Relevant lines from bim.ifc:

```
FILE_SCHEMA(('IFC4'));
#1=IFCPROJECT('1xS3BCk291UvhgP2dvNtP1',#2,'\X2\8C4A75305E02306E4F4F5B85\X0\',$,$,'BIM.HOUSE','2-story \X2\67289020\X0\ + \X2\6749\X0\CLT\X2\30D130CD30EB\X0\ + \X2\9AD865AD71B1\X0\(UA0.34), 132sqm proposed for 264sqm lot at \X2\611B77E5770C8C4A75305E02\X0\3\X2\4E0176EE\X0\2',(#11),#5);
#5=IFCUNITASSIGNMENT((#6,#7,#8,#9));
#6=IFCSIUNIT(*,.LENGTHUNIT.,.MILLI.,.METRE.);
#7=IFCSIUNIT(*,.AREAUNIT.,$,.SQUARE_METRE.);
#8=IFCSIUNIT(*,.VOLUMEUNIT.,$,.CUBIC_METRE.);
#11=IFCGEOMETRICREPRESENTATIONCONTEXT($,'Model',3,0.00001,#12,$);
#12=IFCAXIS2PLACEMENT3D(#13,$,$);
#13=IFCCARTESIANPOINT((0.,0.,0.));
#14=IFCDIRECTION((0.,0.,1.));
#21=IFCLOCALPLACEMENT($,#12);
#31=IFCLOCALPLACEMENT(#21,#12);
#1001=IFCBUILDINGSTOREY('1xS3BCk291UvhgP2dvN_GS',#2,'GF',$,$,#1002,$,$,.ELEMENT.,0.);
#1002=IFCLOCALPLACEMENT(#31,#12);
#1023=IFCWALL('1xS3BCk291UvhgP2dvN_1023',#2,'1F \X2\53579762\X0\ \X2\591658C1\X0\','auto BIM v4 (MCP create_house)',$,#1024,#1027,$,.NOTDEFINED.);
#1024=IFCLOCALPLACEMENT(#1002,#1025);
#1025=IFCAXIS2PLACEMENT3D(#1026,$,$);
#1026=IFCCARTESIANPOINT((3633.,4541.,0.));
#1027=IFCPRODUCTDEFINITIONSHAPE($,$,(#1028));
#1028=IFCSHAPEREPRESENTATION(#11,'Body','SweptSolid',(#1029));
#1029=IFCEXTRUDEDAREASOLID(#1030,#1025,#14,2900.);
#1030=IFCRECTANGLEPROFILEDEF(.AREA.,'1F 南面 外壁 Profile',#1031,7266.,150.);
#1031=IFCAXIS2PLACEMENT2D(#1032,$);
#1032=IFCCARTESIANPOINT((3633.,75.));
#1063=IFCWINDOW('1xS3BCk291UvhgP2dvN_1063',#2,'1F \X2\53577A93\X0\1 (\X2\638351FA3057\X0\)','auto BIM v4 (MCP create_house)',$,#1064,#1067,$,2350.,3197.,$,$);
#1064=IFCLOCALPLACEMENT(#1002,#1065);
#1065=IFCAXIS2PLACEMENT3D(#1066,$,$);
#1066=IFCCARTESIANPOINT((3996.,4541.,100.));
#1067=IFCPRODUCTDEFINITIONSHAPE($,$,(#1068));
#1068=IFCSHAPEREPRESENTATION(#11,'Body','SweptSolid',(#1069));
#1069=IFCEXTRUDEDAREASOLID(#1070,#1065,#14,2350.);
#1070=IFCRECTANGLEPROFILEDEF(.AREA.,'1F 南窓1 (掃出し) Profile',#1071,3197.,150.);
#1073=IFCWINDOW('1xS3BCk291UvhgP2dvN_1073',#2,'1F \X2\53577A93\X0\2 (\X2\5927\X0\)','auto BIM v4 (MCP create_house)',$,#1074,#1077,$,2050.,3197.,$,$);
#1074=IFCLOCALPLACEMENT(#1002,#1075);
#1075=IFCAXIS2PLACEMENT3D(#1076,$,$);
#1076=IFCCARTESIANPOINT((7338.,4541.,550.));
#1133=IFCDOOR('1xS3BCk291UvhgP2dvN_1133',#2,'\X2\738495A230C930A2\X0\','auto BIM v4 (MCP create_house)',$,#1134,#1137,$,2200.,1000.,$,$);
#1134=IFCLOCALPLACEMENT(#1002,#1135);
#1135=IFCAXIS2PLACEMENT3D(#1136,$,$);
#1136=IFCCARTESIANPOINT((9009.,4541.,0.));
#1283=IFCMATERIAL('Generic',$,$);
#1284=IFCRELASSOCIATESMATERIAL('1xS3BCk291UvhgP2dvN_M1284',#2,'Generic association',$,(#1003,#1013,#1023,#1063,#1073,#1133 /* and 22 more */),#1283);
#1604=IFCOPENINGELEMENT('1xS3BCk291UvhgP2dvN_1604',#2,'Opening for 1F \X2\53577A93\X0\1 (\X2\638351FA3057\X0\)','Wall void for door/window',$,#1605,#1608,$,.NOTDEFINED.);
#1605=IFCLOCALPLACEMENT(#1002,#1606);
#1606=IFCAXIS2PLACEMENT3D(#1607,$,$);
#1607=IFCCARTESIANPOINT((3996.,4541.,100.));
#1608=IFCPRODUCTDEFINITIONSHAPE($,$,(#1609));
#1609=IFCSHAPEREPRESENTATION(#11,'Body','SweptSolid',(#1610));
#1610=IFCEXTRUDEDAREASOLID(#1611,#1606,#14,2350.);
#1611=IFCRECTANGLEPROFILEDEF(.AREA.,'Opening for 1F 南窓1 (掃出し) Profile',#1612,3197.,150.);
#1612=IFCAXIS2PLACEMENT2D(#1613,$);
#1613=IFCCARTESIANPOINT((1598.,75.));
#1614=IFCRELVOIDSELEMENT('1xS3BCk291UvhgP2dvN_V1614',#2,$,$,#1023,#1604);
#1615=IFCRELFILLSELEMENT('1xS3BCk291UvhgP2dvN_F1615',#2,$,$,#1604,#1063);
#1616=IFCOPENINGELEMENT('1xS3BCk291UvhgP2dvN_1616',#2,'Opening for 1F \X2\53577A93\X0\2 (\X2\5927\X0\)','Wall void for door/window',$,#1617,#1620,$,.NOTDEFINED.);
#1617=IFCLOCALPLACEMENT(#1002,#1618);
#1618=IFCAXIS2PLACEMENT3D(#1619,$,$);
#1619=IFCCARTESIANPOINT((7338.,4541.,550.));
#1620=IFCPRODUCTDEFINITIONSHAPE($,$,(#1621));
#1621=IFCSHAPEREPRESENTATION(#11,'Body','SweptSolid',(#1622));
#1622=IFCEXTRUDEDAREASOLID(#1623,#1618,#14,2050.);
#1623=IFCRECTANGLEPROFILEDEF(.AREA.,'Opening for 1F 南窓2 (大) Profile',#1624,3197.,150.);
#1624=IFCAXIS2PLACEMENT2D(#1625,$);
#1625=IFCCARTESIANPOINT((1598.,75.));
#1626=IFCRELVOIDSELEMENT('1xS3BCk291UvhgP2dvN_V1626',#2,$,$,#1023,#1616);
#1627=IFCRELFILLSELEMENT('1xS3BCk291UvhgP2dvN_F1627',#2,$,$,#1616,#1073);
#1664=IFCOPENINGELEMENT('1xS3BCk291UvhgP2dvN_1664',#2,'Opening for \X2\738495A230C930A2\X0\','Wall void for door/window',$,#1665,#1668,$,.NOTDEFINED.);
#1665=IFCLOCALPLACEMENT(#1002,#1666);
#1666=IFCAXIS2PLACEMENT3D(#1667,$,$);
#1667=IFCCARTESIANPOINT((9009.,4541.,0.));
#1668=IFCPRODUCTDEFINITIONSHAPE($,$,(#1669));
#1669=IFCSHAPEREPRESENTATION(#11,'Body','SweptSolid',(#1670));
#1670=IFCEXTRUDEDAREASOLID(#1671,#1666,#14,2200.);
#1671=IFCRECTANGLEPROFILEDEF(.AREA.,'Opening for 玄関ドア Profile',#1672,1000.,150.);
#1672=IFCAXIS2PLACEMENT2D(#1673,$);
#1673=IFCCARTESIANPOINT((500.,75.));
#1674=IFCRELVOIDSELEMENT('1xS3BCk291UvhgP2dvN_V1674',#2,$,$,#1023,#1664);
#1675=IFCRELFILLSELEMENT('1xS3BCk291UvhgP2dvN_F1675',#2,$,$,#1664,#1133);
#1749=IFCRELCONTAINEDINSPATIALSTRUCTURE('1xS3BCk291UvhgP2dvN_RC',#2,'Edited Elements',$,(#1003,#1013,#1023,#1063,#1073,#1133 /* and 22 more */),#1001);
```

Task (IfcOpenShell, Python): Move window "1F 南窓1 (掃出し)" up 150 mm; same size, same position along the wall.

```python
import numpy as np
import ifcopenshell
import ifcopenshell.api.geometry
import ifcopenshell.util.placement
import ifcopenshell.util.unit

model = ifcopenshell.open("bim.ifc")
unit_scale = ifcopenshell.util.unit.calculate_unit_scale(model)

window = model.by_guid("1xS3BCk291UvhgP2dvN_1063")
opening = window.FillsVoids[0].RelatingOpeningElement
dz = 0.15 / unit_scale

shift = np.array([0.0, 0.0, dz])
# The window is not placed relative to its opening, so move both.
for product in (opening, window):
    matrix = ifcopenshell.util.placement.get_local_placement(product.ObjectPlacement)
    matrix[:3, 3] += shift
    ifcopenshell.api.geometry.edit_object_placement(model, product=product, matrix=matrix, is_si=False)

print(f"moved by {dz * unit_scale:+.3f} m")

model.write("bim_edited.ifc")
```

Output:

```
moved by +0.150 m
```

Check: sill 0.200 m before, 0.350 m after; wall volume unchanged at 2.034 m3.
